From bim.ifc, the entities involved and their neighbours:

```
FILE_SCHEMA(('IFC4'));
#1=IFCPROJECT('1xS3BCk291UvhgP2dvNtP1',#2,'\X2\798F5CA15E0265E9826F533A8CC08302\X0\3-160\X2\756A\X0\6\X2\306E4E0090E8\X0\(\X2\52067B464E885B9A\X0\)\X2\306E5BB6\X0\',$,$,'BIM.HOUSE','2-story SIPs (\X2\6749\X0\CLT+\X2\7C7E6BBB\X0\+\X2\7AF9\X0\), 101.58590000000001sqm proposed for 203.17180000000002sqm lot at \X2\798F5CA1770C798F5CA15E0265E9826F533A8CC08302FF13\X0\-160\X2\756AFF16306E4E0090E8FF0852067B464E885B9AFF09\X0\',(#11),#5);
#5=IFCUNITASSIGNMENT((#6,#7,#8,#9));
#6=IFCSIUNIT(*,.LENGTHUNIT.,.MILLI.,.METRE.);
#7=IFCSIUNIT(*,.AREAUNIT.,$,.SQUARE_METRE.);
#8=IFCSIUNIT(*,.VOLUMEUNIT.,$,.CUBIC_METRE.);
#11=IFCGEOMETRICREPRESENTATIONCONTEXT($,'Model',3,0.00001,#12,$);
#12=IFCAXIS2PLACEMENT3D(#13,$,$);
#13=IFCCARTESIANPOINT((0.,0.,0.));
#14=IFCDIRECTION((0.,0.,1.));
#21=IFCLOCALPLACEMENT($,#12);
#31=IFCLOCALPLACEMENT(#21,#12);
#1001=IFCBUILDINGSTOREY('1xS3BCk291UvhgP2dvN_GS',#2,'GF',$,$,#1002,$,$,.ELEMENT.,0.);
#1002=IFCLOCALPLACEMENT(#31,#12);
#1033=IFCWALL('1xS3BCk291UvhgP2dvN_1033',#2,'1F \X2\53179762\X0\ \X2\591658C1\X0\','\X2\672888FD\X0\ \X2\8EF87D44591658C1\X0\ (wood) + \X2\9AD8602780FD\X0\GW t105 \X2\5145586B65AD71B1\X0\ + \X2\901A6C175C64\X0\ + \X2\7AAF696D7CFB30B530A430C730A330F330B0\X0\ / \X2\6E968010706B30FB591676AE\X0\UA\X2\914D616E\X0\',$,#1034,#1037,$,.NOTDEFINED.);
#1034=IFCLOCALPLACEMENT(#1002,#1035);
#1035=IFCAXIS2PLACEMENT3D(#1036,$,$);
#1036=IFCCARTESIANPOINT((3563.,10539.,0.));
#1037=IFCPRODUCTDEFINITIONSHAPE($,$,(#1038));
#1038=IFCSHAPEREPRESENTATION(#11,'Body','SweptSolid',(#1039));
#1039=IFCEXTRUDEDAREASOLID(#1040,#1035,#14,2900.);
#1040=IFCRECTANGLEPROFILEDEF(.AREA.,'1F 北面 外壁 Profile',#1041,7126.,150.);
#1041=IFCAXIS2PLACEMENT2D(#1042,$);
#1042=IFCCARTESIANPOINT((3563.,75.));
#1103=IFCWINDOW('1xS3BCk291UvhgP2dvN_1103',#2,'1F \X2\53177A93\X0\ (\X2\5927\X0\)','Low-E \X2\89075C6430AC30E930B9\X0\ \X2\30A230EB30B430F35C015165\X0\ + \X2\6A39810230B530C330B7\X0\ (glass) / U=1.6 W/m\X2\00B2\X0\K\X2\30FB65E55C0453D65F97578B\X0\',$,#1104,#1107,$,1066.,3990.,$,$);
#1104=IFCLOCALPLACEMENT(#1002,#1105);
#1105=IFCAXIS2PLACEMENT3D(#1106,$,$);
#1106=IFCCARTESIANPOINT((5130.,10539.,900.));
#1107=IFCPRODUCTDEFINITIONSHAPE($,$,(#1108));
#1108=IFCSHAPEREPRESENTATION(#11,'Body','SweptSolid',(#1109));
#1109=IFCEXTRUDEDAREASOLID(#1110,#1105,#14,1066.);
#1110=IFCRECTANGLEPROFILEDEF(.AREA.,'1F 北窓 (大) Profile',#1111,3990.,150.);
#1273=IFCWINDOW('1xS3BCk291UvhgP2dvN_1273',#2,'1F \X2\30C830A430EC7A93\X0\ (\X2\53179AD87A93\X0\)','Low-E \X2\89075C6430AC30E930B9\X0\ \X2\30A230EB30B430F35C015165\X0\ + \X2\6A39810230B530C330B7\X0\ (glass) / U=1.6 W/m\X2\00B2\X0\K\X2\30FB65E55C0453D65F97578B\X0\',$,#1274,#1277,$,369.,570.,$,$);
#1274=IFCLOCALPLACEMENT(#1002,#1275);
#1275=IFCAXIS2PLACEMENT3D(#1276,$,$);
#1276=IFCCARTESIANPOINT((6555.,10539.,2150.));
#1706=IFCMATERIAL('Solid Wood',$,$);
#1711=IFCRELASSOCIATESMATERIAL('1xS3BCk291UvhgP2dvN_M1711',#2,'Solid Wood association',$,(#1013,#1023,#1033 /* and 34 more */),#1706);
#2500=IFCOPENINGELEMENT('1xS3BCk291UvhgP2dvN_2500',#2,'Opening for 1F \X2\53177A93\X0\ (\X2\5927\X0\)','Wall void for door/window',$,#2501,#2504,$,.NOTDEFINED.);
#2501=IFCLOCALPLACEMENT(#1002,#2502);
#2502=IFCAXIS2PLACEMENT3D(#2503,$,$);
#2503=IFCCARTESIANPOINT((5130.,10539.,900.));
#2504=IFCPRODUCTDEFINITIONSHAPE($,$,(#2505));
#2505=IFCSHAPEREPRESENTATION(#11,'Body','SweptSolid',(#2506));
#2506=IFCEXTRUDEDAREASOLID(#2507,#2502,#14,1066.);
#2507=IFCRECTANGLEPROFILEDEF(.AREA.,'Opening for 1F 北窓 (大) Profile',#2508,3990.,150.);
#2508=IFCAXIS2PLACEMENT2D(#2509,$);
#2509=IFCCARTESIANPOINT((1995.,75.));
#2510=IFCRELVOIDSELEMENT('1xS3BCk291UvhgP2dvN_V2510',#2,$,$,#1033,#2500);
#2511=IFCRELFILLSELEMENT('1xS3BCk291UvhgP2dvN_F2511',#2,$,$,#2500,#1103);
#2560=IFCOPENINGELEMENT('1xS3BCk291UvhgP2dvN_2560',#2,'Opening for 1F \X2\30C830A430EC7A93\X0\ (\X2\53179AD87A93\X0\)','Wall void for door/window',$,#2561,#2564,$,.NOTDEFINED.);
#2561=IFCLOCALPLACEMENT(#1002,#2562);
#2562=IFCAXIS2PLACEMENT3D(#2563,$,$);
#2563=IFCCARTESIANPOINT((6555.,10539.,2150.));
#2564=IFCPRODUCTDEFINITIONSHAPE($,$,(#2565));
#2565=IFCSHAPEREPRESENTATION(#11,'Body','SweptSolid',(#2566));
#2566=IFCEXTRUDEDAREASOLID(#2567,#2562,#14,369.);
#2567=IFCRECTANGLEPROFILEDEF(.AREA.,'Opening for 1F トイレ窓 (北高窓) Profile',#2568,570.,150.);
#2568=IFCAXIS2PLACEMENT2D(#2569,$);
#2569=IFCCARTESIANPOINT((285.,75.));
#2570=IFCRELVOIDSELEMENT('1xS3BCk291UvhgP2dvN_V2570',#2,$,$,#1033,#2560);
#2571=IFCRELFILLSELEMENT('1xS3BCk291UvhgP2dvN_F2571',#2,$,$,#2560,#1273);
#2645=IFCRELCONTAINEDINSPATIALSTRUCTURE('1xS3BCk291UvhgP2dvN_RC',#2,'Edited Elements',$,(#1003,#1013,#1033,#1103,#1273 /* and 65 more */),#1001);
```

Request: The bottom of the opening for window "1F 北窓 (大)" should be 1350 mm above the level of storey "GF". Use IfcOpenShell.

```python
import numpy as np
import ifcopenshell
import ifcopenshell.api.geometry
import ifcopenshell.geom
import ifcopenshell.util.element
import ifcopenshell.util.placement
import ifcopenshell.util.shape
import ifcopenshell.util.unit

model = ifcopenshell.open("bim.ifc")
unit_scale = ifcopenshell.util.unit.calculate_unit_scale(model)

window = model.by_guid("1xS3BCk291UvhgP2dvN_1103")
opening = window.FillsVoids[0].RelatingOpeningElement
storey = ifcopenshell.util.element.get_container(window, ifc_class="IfcBuildingStorey")
level = ifcopenshell.util.placement.get_local_placement(storey.ObjectPlacement)[2, 3]

# The opening's origin need not be at the sill, so measure its lowest point.
shape = ifcopenshell.geom.create_shape(ifcopenshell.geom.settings(), opening)
bottom = ifcopenshell.util.shape.get_shape_bottom_elevation(shape, shape.geometry) / unit_scale
dz = level + 1350.0 - bottom

shift = np.array([0.0, 0.0, dz])
# The window is not placed relative to its opening, so move both.
for product in (opening, window):
    matrix = ifcopenshell.util.placement.get_local_placement(product.ObjectPlacement)
    matrix[:3, 3] += shift
    ifcopenshell.api.geometry.edit_object_placement(model, product=product, matrix=matrix, is_si=False)

print(f"moved by {dz * unit_scale:+.3f} m")

model.write("bim_v2.ifc")
```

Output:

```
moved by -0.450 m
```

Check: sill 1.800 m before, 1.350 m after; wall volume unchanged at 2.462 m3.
